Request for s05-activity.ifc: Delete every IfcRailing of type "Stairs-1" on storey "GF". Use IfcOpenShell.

First a look at what the model holds.

```python
import ifcopenshell
import ifcopenshell.util.element

model = ifcopenshell.open("s05-activity.ifc")
print(model.schema)
storey = next(s for s in model.by_type("IfcBuildingStorey") if s.Name == "GF")
railings = [e for e in ifcopenshell.util.element.get_decomposition(storey) if e.is_a("IfcRailing")]
seen = {}
for e in railings:
    element_type = ifcopenshell.util.element.get_type(e)
    name = element_type.Name if element_type not in (None, e) else None
    seen[name] = seen.get(name, 0) + 1
for name, count in sorted(seen.items(), key=str):
    print(count, "x", name)
```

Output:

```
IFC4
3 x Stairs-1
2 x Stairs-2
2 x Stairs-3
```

```python
import ifcopenshell
import ifcopenshell.api.root
import ifcopenshell.util.element

model = ifcopenshell.open("s05-activity.ifc")

storey = next(s for s in model.by_type("IfcBuildingStorey") if s.Name == "GF")
railings = [e for e in ifcopenshell.util.element.get_decomposition(storey) if e.is_a("IfcRailing")]
targets = [e for e in railings if (t := ifcopenshell.util.element.get_type(e)) not in (None, e) and t.Name == "Stairs-1"]

for e in targets:
    ifcopenshell.api.root.remove_product(model, product=e)
print(len(targets), "removed")

model.write("s05-activity-out.ifc")
```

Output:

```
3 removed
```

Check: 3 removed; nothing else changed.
